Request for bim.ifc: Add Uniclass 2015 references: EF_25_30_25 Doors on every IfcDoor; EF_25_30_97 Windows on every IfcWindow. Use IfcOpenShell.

First a look at what the model holds.

```python
import ifcopenshell

model = ifcopenshell.open("bim.ifc")
print(model.schema)
print("classifications:", [c.Name for c in model.by_type("IfcClassification")])
for ifc_class in ("IfcDoor", "IfcRoof", "IfcStair", "IfcWall", "IfcWindow"):
    print(ifc_class, len(model.by_type(ifc_class)))
```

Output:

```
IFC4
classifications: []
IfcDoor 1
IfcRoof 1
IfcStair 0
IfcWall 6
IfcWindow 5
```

```python
import ifcopenshell
import ifcopenshell.api.classification

model = ifcopenshell.open("bim.ifc")

system = ifcopenshell.api.classification.add_classification(model, classification="Uniclass 2015")

codes = {
    "IfcDoor": ("EF_25_30_25", "Doors"),
    "IfcWindow": ("EF_25_30_97", "Windows"),
}
for ifc_class, (code, name) in codes.items():
    products = model.by_type(ifc_class)
    ifcopenshell.api.classification.add_reference(
        model, products=products, classification=system, identification=code, name=name
    )
    print(code, len(products))

model.write("bim_edited.ifc")
```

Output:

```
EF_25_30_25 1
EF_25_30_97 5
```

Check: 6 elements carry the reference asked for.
